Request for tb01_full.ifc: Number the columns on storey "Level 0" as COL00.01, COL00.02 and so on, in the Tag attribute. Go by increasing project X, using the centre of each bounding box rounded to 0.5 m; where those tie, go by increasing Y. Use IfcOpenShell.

First a look at what the model holds.

```python
import ifcopenshell
import ifcopenshell.util.element
import ifcopenshell.util.placement

model = ifcopenshell.open("tb01_full.ifc")
print(model.schema)
storey = next(s for s in model.by_type("IfcBuildingStorey") if s.Name == "Level 0")
columns = [e for e in ifcopenshell.util.element.get_decomposition(storey) if e.is_a("IfcColumn")]
for e in sorted(columns, key=lambda e: e.id()):
    origin = ifcopenshell.util.placement.get_local_placement(e.ObjectPlacement)[:3, 3]
    print(e.id(), e.Tag, e.Name, origin.round(2) + 0.0, sep=" | ")
```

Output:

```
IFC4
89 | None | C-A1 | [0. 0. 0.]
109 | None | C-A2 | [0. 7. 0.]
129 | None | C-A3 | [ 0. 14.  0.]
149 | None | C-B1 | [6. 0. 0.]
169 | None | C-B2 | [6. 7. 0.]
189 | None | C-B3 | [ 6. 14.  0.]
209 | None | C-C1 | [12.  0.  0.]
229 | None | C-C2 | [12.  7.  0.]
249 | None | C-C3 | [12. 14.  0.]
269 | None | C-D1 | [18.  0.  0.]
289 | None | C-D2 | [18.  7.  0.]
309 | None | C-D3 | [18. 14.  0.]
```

```python
import ifcopenshell
import ifcopenshell.geom
import ifcopenshell.util.element
import ifcopenshell.util.shape

model = ifcopenshell.open("tb01_full.ifc")
settings = ifcopenshell.geom.settings()
settings.set("use-world-coords", True)


def centre(element):
    shape = ifcopenshell.geom.create_shape(settings, element)
    return ifcopenshell.util.shape.get_bbox_centroid(shape.geometry)


storey = next(s for s in model.by_type("IfcBuildingStorey") if s.Name == "Level 0")
columns = [e for e in ifcopenshell.util.element.get_decomposition(storey) if e.is_a("IfcColumn")]

# Insertion points can sit at a corner or the storey origin, so sort by the geometry (in metres).
centres = {e: centre(e) for e in columns}
columns.sort(key=lambda e: (round(centres[e][0] / 0.5), centres[e][1]))

for i, e in enumerate(columns, start=1):
    number = f"COL00.{i:02d}"
    e.Tag = number
    print(e.id(), number)

model.write("tb01_full_updated.ifc")
```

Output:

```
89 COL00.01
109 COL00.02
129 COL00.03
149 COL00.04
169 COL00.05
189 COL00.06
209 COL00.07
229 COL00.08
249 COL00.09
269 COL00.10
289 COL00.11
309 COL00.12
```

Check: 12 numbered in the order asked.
